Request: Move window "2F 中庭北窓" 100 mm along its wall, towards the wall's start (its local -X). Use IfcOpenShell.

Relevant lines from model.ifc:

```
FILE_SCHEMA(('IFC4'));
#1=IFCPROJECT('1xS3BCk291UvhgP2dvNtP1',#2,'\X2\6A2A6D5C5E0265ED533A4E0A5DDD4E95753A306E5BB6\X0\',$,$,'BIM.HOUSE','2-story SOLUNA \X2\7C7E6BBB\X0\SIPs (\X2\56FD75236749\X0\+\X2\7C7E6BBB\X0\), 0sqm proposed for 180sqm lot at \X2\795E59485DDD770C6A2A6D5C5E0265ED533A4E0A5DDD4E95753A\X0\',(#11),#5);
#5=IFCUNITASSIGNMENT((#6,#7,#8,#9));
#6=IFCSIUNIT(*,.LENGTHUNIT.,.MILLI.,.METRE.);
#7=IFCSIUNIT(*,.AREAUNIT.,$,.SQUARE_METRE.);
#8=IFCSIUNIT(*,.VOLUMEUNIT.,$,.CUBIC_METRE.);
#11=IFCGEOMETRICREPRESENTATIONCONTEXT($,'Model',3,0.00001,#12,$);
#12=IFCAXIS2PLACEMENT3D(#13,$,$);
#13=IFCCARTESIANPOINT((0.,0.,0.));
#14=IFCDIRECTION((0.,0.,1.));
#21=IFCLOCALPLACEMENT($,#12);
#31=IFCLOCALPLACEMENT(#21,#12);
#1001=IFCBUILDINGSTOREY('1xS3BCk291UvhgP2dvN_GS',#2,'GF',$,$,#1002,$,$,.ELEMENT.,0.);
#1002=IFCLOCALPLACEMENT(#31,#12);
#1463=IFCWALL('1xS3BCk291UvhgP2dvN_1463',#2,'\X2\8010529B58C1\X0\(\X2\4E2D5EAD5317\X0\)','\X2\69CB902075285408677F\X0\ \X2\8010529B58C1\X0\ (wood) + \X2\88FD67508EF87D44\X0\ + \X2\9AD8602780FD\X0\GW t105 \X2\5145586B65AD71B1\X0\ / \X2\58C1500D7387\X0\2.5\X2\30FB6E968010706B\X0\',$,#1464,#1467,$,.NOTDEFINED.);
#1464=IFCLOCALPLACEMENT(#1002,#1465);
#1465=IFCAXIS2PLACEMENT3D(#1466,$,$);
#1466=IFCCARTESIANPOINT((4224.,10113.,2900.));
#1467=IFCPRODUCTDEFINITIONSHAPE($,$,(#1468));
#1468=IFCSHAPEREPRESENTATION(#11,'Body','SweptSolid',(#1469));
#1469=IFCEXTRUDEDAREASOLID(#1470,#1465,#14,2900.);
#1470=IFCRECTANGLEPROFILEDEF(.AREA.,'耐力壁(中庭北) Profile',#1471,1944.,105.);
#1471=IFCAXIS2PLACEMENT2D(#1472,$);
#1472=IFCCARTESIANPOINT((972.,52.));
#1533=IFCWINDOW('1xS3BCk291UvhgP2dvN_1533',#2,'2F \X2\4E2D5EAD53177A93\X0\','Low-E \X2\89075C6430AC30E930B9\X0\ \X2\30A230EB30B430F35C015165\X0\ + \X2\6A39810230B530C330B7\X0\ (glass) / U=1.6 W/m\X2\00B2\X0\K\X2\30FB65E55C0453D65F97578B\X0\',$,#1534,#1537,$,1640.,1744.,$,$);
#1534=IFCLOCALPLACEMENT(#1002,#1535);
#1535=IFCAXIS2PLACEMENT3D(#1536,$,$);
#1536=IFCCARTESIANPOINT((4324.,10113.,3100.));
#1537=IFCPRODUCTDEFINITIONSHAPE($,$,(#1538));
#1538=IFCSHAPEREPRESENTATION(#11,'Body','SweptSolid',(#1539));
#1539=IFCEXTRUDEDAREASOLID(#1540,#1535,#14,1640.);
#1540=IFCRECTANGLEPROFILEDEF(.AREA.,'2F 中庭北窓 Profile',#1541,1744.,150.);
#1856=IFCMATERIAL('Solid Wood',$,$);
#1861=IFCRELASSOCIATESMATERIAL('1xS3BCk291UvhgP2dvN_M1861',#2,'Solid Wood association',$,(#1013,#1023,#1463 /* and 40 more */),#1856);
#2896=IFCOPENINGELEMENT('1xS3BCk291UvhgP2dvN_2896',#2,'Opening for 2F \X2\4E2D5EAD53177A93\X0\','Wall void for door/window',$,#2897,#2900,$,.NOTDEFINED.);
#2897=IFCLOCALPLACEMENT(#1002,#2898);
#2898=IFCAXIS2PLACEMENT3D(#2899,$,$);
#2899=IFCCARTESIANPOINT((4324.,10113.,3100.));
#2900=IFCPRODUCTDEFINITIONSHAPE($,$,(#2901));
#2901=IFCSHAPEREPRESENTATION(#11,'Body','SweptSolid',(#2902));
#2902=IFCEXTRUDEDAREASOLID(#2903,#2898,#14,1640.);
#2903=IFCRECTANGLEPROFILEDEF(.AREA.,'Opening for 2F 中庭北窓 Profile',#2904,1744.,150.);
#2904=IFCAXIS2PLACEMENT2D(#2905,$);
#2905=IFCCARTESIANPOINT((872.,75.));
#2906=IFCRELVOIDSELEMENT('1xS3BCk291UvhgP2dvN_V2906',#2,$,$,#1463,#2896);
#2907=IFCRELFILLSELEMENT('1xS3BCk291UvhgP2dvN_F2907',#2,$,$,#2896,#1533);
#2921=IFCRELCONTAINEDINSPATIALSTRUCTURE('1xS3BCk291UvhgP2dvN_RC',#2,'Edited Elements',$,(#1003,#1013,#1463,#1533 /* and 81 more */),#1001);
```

```python
import ifcopenshell
import ifcopenshell.api.geometry
import ifcopenshell.util.placement
import ifcopenshell.util.unit

model = ifcopenshell.open("model.ifc")
unit_scale = ifcopenshell.util.unit.calculate_unit_scale(model)

window = model.by_guid("1xS3BCk291UvhgP2dvN_1533")
opening = window.FillsVoids[0].RelatingOpeningElement
wall = opening.VoidsElements[0].RelatingBuildingElement

wall_matrix = ifcopenshell.util.placement.get_local_placement(wall.ObjectPlacement)
shift = wall_matrix[:3, 0] * -0.1 / unit_scale
before = ifcopenshell.util.placement.get_local_placement(window.ObjectPlacement)[:3, 3].copy()

# The window is not placed relative to its opening, so move both.
for product in (opening, window):
    matrix = ifcopenshell.util.placement.get_local_placement(product.ObjectPlacement)
    matrix[:3, 3] += shift
    ifcopenshell.api.geometry.edit_object_placement(model, product=product, matrix=matrix, is_si=False)

after = ifcopenshell.util.placement.get_local_placement(window.ObjectPlacement)[:3, 3]
print("window moved by", (after - before).round(3) + 0.0)

model.write("model_rev.ifc")
```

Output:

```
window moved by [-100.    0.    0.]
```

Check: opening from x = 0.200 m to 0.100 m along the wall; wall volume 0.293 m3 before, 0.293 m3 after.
